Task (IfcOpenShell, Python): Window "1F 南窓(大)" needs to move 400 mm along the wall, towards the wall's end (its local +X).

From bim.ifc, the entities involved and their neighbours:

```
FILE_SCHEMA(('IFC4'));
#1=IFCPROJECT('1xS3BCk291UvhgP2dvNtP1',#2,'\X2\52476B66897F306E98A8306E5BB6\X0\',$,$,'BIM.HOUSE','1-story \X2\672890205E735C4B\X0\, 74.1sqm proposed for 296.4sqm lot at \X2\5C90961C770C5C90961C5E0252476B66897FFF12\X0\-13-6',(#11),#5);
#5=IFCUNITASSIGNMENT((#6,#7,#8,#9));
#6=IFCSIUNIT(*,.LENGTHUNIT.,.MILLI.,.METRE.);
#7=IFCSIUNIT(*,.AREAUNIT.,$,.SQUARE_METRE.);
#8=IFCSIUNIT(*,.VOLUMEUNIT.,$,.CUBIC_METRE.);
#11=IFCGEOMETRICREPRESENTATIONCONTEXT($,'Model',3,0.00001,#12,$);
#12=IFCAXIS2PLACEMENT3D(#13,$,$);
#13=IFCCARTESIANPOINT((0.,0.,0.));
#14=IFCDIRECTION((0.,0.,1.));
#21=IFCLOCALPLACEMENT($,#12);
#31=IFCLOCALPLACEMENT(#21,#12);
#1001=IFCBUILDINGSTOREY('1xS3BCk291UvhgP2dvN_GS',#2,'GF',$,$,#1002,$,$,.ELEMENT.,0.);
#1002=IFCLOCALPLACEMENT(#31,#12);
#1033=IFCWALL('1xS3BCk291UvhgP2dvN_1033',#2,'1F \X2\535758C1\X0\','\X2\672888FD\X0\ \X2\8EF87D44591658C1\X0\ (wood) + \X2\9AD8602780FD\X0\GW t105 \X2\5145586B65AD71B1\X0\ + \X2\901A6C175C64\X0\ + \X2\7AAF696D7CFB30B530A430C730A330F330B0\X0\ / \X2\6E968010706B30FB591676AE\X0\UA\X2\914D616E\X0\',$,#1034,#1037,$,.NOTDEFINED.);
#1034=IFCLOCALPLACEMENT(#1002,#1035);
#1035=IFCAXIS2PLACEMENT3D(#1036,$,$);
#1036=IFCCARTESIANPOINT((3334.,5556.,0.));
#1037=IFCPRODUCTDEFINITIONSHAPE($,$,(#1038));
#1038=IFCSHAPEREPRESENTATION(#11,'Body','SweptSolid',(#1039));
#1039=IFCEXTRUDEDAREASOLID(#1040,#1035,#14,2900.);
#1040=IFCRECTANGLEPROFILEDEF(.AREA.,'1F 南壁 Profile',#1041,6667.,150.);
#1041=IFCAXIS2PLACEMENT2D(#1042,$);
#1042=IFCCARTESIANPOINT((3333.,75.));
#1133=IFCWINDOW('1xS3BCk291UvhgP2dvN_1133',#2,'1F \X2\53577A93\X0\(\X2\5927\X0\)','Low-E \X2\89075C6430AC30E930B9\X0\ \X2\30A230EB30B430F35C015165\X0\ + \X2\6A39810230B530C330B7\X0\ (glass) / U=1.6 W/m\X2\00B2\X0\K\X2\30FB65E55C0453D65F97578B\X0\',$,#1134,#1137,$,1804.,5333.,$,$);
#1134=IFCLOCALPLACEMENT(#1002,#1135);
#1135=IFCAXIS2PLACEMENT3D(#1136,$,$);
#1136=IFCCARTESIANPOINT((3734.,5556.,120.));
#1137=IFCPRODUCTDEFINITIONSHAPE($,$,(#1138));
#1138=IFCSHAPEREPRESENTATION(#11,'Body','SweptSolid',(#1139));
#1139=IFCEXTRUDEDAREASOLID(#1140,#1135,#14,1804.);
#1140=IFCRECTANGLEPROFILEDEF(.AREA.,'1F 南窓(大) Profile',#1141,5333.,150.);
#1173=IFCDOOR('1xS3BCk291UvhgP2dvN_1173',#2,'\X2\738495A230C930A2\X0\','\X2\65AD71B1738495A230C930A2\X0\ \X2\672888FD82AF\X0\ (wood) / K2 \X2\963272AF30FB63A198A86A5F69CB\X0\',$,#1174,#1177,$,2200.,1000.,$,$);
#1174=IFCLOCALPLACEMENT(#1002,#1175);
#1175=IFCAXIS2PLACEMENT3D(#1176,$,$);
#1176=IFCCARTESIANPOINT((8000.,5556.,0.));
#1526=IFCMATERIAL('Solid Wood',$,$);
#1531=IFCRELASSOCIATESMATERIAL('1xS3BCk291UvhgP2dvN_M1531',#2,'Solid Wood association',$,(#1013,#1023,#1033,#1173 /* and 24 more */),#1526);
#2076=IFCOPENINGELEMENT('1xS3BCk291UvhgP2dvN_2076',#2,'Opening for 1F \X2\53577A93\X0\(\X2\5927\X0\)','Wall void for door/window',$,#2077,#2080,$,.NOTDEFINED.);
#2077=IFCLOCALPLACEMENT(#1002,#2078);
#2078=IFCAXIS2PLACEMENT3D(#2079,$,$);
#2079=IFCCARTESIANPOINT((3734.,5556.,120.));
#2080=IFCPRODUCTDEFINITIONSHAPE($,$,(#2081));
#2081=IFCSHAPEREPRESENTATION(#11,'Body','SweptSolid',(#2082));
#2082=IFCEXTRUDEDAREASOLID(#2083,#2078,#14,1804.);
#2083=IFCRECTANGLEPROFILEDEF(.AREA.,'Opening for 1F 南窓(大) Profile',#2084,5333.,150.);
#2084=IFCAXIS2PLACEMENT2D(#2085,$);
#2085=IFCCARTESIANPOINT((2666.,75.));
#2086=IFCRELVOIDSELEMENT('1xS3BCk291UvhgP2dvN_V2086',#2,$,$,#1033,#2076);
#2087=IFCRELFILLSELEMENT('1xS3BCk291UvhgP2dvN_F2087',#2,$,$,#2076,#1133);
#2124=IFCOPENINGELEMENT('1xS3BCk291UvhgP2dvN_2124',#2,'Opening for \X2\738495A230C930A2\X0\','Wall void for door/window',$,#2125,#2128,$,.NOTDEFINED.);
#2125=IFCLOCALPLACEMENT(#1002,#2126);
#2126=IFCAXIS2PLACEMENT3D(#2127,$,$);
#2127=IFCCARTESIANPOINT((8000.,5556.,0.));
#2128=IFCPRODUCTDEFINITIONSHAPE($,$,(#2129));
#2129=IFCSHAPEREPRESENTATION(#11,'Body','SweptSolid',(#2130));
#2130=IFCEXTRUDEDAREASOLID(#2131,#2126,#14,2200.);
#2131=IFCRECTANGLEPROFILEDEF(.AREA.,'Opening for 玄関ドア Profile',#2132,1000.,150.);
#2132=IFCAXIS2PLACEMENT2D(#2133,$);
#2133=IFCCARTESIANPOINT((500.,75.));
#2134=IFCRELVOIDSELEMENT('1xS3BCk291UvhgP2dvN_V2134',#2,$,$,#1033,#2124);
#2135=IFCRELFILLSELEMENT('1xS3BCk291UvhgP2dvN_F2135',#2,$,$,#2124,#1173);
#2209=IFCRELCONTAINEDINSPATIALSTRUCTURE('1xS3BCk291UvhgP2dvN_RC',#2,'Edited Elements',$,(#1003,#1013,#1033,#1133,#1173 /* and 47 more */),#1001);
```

```python
import ifcopenshell
import ifcopenshell.api.geometry
import ifcopenshell.util.placement
import ifcopenshell.util.unit

model = ifcopenshell.open("bim.ifc")
unit_scale = ifcopenshell.util.unit.calculate_unit_scale(model)

window = model.by_guid("1xS3BCk291UvhgP2dvN_1133")
opening = window.FillsVoids[0].RelatingOpeningElement
wall = opening.VoidsElements[0].RelatingBuildingElement

wall_matrix = ifcopenshell.util.placement.get_local_placement(wall.ObjectPlacement)
shift = wall_matrix[:3, 0] * 0.4 / unit_scale
before = ifcopenshell.util.placement.get_local_placement(window.ObjectPlacement)[:3, 3].copy()

# The window is not placed relative to its opening, so move both.
for product in (opening, window):
    matrix = ifcopenshell.util.placement.get_local_placement(product.ObjectPlacement)
    matrix[:3, 3] += shift
    ifcopenshell.api.geometry.edit_object_placement(model, product=product, matrix=matrix, is_si=False)

after = ifcopenshell.util.placement.get_local_placement(window.ObjectPlacement)[:3, 3]
print("window moved by", (after - before).round(3) + 0.0)

model.write("bim_updated.ifc")
```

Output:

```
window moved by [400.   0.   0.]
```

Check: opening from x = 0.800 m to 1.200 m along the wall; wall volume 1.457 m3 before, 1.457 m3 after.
